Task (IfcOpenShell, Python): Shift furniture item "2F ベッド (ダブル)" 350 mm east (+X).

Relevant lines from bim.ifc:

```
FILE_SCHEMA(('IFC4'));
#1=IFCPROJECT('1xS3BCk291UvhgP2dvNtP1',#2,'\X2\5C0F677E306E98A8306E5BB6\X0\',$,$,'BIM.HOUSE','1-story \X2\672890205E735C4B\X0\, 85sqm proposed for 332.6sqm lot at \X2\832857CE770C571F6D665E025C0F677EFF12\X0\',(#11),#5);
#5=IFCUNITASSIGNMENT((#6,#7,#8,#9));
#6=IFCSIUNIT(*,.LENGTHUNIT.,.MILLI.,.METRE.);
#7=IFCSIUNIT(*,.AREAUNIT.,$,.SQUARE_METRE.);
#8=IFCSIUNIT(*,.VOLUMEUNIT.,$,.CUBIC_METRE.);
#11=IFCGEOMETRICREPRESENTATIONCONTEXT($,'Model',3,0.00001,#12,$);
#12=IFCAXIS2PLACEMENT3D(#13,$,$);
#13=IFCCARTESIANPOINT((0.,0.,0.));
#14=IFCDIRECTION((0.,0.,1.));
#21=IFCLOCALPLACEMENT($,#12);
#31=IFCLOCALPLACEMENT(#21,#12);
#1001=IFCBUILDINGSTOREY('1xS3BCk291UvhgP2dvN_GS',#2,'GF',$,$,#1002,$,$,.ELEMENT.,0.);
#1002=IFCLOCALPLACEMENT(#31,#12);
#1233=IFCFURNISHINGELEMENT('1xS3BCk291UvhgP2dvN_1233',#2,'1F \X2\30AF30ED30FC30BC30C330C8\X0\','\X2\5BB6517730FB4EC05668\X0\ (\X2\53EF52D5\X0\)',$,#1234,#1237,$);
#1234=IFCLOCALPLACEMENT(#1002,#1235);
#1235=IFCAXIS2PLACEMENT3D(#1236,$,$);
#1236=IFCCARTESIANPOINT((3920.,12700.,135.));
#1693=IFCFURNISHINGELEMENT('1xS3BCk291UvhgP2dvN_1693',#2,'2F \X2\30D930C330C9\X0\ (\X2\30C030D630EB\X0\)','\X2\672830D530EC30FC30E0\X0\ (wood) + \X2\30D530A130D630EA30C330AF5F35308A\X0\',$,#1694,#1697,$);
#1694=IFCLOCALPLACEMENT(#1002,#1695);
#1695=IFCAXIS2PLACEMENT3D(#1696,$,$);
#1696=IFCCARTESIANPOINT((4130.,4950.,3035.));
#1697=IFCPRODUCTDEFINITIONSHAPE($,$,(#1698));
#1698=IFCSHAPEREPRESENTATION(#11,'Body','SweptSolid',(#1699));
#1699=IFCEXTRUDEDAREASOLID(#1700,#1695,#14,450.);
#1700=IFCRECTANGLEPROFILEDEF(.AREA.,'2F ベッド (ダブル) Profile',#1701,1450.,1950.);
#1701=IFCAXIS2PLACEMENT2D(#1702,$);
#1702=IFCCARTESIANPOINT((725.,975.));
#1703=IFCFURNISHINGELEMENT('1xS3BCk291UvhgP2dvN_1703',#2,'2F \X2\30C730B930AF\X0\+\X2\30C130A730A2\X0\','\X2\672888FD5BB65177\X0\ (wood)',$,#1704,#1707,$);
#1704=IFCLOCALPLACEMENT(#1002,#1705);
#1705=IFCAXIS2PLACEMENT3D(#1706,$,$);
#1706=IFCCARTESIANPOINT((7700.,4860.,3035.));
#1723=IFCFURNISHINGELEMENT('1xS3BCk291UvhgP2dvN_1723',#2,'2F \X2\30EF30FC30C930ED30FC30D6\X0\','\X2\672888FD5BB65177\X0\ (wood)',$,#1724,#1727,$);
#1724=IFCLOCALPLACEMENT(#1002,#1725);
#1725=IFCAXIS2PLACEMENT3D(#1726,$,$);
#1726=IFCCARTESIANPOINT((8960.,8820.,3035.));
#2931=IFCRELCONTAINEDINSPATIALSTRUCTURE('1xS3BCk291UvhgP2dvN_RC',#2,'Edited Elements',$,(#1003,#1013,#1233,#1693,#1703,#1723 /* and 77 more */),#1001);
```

```python
import ifcopenshell
import ifcopenshell.api.geometry
import ifcopenshell.util.placement

model = ifcopenshell.open("bim.ifc")

item = model.by_id(1693)
matrix = ifcopenshell.util.placement.get_local_placement(item.ObjectPlacement)
matrix[0, 3] += 350.0
ifcopenshell.api.geometry.edit_object_placement(model, product=item, matrix=matrix, is_si=False)

print(ifcopenshell.util.placement.get_local_placement(item.ObjectPlacement).round(3) + 0.0)

model.write("bim_edited.ifc")
```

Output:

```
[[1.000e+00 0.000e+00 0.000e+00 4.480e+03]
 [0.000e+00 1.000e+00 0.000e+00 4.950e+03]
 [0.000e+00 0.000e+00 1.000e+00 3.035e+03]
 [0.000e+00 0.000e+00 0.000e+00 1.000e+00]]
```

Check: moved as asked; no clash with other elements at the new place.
